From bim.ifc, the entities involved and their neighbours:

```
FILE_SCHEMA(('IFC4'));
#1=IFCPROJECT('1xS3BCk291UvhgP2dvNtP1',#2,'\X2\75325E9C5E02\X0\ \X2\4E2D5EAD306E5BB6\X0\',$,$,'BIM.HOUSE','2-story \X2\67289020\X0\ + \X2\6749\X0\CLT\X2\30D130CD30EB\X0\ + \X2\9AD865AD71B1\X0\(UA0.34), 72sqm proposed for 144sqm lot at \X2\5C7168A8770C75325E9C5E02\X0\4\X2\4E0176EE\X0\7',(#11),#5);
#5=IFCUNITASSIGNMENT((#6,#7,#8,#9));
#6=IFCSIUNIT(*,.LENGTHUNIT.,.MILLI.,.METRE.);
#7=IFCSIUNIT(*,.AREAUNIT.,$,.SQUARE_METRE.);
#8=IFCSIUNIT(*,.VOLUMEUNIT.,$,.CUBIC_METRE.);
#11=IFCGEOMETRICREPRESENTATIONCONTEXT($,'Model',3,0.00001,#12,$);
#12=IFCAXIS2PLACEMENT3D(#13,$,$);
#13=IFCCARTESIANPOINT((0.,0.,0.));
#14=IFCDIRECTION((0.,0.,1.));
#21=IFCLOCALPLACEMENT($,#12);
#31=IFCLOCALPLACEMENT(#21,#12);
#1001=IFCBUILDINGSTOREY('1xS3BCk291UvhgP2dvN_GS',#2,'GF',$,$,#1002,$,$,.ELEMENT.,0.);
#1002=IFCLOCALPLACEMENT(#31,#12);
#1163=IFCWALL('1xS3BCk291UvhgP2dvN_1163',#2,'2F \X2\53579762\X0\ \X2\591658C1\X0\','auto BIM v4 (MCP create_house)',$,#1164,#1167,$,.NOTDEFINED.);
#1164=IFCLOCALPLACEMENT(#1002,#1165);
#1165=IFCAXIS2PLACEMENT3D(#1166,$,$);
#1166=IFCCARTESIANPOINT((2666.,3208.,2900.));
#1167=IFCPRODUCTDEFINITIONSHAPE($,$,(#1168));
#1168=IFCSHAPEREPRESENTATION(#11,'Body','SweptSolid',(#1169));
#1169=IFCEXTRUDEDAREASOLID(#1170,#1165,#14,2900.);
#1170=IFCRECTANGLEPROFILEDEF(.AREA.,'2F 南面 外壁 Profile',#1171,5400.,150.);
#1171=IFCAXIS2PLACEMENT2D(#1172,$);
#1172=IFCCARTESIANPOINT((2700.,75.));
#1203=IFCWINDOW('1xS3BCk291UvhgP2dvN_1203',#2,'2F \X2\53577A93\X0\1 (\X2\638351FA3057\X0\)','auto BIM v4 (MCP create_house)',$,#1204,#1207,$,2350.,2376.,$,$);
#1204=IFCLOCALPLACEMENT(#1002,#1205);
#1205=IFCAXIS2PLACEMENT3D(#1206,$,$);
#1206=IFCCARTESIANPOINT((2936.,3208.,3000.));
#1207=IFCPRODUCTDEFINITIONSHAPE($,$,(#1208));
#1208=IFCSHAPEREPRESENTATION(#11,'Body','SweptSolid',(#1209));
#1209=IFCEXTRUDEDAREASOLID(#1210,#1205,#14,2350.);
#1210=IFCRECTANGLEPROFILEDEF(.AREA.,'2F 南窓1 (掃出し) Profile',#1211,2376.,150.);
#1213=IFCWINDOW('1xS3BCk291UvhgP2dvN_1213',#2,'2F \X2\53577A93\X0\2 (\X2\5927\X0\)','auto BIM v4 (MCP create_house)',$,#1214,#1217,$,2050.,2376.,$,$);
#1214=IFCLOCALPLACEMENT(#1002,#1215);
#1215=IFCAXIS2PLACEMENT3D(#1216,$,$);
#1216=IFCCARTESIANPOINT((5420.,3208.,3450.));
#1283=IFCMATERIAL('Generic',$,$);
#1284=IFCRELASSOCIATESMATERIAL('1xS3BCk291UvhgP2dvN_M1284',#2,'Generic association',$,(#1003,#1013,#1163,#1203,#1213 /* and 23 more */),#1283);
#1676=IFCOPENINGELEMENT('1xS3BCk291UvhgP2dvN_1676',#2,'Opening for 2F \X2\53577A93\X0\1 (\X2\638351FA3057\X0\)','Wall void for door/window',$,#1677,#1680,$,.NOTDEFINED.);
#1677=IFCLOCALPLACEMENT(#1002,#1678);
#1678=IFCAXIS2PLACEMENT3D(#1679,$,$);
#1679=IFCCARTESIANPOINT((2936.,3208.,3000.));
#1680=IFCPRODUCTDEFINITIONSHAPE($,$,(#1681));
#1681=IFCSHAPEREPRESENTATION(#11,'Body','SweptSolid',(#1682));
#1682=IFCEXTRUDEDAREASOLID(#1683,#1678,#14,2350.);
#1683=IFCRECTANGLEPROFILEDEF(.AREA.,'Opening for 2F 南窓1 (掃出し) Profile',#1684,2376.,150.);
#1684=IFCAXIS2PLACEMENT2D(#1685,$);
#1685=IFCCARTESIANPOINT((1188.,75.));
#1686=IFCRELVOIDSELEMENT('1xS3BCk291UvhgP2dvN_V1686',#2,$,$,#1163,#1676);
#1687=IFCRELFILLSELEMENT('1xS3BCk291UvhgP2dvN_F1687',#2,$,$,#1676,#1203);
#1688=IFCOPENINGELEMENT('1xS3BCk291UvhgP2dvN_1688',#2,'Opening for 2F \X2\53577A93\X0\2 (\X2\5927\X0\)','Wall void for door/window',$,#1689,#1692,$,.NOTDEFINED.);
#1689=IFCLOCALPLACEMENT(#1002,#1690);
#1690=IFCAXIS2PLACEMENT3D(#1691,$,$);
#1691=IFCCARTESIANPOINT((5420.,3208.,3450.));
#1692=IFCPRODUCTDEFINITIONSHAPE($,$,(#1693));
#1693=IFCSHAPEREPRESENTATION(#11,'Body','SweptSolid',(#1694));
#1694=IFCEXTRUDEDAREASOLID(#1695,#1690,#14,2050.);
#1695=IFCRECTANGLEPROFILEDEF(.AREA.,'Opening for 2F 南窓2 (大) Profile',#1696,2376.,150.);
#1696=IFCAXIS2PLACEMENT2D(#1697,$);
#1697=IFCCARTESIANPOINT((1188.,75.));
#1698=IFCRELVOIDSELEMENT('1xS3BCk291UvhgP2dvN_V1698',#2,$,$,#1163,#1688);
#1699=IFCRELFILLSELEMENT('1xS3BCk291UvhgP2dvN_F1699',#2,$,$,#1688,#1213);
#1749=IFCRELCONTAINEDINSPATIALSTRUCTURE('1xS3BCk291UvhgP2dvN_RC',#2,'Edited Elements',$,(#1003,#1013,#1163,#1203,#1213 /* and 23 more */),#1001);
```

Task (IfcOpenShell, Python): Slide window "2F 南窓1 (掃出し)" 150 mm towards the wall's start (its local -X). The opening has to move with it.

```python
import ifcopenshell
import ifcopenshell.api.geometry
import ifcopenshell.util.placement
import ifcopenshell.util.unit

model = ifcopenshell.open("bim.ifc")
unit_scale = ifcopenshell.util.unit.calculate_unit_scale(model)

window = model.by_guid("1xS3BCk291UvhgP2dvN_1203")
opening = window.FillsVoids[0].RelatingOpeningElement
wall = opening.VoidsElements[0].RelatingBuildingElement

wall_matrix = ifcopenshell.util.placement.get_local_placement(wall.ObjectPlacement)
shift = wall_matrix[:3, 0] * -0.15 / unit_scale
before = ifcopenshell.util.placement.get_local_placement(window.ObjectPlacement)[:3, 3].copy()

# The window is not placed relative to its opening, so move both.
for product in (opening, window):
    matrix = ifcopenshell.util.placement.get_local_placement(product.ObjectPlacement)
    matrix[:3, 3] += shift
    ifcopenshell.api.geometry.edit_object_placement(model, product=product, matrix=matrix, is_si=False)

after = ifcopenshell.util.placement.get_local_placement(window.ObjectPlacement)[:3, 3]
print("window moved by", (after - before).round(3) + 0.0)

model.write("bim-out.ifc")
```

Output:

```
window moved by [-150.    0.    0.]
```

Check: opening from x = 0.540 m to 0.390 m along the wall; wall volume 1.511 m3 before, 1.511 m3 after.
